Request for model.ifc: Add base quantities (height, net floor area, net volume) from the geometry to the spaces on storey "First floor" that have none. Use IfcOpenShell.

First a look at what the model holds.

```python
import ifcopenshell
import ifcopenshell.util.element
import ifcopenshell.util.unit

model = ifcopenshell.open("model.ifc")
print(model.schema)
for unit_type in ("LENGTHUNIT", "AREAUNIT", "VOLUMEUNIT"):
    print(unit_type, ifcopenshell.util.unit.calculate_unit_scale(model, unit_type))
storey = next(s for s in model.by_type("IfcBuildingStorey") if s.Name == "First floor")
spaces = [e for e in ifcopenshell.util.element.get_decomposition(storey) if e.is_a("IfcSpace")]
for e in sorted(spaces, key=lambda e: e.id()):
    print(e.id(), e.is_a(), e.Name, list(ifcopenshell.util.element.get_psets(e, qtos_only=True)), sep=" | ")
```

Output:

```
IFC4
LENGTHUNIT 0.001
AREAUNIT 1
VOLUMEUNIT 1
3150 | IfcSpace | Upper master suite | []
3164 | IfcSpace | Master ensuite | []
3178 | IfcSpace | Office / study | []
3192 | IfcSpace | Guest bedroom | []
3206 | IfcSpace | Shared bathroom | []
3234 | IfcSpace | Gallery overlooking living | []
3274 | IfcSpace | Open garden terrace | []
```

```python
import ifcopenshell
import ifcopenshell.api.pset
import ifcopenshell.geom
import ifcopenshell.util.element
import ifcopenshell.util.shape
import ifcopenshell.util.unit

model = ifcopenshell.open("model.ifc")
unit_scale = ifcopenshell.util.unit.calculate_unit_scale(model)
area_scale = ifcopenshell.util.unit.calculate_unit_scale(model, "AREAUNIT")
volume_scale = ifcopenshell.util.unit.calculate_unit_scale(model, "VOLUMEUNIT")
settings = ifcopenshell.geom.settings()

storey = next(s for s in model.by_type("IfcBuildingStorey") if s.Name == "First floor")
spaces = [e for e in ifcopenshell.util.element.get_decomposition(storey) if e.is_a("IfcSpace")]

for e in sorted(spaces, key=lambda e: e.id()):
    if ifcopenshell.util.element.get_psets(e, qtos_only=True, should_inherit=False):
        continue
    # Geometry comes back in metres, in the element's own axes.
    shape = ifcopenshell.geom.create_shape(settings, e)
    values = {
        "Height": ifcopenshell.util.shape.get_z(shape.geometry) / unit_scale,
        "NetFloorArea": ifcopenshell.util.shape.get_footprint_area(shape.geometry) / area_scale,
        "NetVolume": ifcopenshell.util.shape.get_volume(shape.geometry) / volume_scale,
    }
    qto = ifcopenshell.api.pset.add_qto(model, product=e, name="Qto_SpaceBaseQuantities")
    ifcopenshell.api.pset.edit_qto(model, qto=qto, properties=values)
    print(e.id(), {k: round(v, 3) for k, v in values.items()})

model.write("model_edited.ifc")
```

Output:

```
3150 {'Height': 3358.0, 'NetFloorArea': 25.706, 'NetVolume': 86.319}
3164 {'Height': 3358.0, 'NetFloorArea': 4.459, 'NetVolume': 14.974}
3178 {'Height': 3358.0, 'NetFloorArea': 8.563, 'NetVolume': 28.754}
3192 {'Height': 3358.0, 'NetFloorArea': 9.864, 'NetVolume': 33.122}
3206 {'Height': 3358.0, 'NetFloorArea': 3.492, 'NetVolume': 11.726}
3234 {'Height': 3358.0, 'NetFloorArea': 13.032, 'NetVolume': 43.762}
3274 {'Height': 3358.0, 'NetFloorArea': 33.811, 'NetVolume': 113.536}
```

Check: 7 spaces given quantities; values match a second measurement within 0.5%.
